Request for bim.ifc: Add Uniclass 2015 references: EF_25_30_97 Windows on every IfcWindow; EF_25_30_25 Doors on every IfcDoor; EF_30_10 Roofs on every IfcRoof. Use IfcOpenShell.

First a look at what the model holds.

```python
import ifcopenshell

model = ifcopenshell.open("bim.ifc")
print(model.schema)
print("classifications:", [c.Name for c in model.by_type("IfcClassification")])
for ifc_class in ("IfcDoor", "IfcRoof", "IfcStair", "IfcWall", "IfcWindow"):
    print(ifc_class, len(model.by_type(ifc_class)))
```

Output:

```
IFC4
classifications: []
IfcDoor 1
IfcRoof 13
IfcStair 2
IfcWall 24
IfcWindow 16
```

```python
import ifcopenshell
import ifcopenshell.api.classification

model = ifcopenshell.open("bim.ifc")

system = ifcopenshell.api.classification.add_classification(model, classification="Uniclass 2015")

codes = {
    "IfcWindow": ("EF_25_30_97", "Windows"),
    "IfcDoor": ("EF_25_30_25", "Doors"),
    "IfcRoof": ("EF_30_10", "Roofs"),
}
for ifc_class, (code, name) in codes.items():
    products = model.by_type(ifc_class)
    ifcopenshell.api.classification.add_reference(
        model, products=products, classification=system, identification=code, name=name
    )
    print(code, len(products))

model.write("bim-out.ifc")
```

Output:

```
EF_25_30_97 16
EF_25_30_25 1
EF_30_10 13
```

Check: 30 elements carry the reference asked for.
